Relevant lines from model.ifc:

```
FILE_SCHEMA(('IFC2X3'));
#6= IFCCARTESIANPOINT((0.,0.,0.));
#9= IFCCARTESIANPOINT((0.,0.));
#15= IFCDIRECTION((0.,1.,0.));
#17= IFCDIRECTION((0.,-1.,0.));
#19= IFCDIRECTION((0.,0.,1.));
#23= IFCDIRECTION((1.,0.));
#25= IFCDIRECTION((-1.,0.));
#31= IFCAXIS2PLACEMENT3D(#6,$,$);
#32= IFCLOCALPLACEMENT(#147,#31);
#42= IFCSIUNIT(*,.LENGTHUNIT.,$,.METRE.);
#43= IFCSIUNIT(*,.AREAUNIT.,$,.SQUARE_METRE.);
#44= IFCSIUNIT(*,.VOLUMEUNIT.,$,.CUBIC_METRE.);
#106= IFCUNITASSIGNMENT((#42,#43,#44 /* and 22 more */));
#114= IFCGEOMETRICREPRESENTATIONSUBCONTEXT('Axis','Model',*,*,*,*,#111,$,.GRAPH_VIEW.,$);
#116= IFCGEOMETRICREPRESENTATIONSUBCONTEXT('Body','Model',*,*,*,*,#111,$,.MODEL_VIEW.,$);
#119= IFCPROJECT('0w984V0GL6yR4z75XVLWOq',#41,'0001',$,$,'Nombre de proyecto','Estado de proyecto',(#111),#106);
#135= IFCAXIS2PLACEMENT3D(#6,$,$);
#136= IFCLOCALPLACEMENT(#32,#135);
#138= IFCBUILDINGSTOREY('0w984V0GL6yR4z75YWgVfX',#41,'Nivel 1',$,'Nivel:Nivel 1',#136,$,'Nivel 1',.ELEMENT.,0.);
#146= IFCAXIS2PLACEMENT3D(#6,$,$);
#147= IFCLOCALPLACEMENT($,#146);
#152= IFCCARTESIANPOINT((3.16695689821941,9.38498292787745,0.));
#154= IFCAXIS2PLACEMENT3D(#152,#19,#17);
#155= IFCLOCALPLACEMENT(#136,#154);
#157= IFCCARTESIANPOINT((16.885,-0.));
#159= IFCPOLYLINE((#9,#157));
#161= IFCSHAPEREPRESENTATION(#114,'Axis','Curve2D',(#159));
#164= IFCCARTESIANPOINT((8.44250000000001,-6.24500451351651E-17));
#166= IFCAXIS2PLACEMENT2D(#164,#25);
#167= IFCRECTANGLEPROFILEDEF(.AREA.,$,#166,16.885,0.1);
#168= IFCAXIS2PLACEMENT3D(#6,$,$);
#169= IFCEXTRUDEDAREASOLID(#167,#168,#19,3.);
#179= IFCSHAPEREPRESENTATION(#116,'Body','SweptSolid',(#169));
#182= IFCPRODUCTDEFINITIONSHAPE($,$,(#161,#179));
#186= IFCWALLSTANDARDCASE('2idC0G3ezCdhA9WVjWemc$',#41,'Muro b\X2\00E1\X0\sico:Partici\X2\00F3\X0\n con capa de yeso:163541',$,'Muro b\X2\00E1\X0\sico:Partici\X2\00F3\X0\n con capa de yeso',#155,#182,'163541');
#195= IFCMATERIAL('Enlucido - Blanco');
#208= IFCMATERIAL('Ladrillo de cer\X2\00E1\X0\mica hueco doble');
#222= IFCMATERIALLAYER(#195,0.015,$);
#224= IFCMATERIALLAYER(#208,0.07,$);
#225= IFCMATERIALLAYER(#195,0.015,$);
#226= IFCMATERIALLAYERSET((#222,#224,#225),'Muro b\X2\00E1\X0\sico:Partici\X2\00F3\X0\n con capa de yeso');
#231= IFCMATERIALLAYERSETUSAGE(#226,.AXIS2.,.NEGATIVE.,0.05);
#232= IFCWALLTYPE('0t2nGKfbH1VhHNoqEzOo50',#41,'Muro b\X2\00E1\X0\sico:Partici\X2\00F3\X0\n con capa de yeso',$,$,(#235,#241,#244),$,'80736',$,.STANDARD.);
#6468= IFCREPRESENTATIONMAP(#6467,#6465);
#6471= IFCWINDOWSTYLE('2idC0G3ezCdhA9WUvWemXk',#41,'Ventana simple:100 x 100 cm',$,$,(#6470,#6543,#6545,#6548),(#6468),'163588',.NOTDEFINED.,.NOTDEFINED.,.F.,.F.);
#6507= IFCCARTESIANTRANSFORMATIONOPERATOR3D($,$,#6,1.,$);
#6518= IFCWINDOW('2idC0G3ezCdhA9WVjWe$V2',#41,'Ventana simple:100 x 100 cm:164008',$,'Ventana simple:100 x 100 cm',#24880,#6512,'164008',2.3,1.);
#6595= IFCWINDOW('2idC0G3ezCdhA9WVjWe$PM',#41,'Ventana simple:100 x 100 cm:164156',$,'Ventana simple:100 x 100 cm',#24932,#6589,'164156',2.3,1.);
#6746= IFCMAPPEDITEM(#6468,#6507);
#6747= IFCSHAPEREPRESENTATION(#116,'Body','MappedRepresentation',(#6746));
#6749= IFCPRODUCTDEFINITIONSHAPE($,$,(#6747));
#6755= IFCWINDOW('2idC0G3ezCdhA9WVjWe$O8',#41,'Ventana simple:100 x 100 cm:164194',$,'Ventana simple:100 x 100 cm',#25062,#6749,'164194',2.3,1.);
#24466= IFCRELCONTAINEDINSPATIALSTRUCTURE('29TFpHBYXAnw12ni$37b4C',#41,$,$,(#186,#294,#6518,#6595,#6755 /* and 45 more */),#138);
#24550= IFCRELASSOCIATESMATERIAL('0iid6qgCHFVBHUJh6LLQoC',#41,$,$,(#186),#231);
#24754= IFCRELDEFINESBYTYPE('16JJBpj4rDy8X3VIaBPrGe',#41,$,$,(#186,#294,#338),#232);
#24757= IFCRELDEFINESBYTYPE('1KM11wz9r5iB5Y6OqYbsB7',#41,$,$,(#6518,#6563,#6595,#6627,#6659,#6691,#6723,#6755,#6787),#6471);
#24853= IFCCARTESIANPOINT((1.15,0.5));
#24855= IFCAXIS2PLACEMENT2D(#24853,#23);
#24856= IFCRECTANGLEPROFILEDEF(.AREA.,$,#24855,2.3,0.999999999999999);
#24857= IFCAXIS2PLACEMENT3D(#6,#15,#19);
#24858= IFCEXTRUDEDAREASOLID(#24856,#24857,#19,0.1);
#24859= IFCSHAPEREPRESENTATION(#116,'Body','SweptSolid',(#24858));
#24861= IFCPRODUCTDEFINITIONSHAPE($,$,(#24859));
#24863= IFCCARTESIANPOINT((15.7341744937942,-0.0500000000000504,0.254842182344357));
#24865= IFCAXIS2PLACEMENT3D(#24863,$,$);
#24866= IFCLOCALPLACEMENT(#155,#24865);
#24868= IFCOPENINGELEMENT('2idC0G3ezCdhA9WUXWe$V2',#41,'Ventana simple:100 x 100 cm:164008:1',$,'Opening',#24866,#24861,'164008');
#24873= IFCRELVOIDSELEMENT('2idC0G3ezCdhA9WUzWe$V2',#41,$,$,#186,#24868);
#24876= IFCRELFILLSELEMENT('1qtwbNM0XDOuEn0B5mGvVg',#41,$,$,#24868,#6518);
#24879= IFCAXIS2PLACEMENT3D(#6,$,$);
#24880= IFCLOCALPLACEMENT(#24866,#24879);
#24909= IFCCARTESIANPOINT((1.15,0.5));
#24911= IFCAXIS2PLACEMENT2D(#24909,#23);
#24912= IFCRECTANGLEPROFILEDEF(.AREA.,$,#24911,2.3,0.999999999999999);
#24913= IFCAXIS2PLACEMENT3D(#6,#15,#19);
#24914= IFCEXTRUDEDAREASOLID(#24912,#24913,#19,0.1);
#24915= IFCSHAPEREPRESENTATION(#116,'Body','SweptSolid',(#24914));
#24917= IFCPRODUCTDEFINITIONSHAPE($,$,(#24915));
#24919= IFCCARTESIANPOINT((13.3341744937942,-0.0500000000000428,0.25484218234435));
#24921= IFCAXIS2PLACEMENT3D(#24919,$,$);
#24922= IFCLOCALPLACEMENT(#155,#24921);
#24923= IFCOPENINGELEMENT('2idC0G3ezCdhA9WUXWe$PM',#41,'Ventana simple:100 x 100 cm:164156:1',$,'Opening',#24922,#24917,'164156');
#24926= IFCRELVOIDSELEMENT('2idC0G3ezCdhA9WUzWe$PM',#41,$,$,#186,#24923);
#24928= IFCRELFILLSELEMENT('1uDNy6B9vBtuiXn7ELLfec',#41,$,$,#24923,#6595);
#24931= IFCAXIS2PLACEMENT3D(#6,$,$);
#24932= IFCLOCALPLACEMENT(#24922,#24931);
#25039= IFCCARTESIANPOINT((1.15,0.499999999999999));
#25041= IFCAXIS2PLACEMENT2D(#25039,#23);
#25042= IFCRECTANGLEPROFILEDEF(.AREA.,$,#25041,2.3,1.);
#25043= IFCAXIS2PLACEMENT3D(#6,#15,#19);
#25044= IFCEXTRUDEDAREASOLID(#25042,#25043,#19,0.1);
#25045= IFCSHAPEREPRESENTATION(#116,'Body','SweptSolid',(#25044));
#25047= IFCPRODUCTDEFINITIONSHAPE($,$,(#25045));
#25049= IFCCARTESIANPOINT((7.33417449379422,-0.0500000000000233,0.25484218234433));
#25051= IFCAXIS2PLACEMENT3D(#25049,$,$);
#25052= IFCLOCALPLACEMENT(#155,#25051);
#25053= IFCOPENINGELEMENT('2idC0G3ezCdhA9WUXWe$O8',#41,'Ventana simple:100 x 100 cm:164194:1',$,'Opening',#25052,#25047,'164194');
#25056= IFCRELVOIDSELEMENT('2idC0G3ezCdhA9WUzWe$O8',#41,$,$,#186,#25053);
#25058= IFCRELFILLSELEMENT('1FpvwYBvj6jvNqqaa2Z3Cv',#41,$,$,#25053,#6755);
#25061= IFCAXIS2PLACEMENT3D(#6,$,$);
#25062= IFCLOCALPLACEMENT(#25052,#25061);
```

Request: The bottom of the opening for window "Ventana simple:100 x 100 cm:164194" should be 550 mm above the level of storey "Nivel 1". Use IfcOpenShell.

```python
import numpy as np
import ifcopenshell
import ifcopenshell.api.geometry
import ifcopenshell.geom
import ifcopenshell.util.element
import ifcopenshell.util.placement
import ifcopenshell.util.shape
import ifcopenshell.util.unit

model = ifcopenshell.open("model.ifc")
unit_scale = ifcopenshell.util.unit.calculate_unit_scale(model)

window = model.by_guid("2idC0G3ezCdhA9WVjWe$O8")
opening = window.FillsVoids[0].RelatingOpeningElement
storey = ifcopenshell.util.element.get_container(window, ifc_class="IfcBuildingStorey")
level = ifcopenshell.util.placement.get_local_placement(storey.ObjectPlacement)[2, 3]

# The opening's origin need not be at the sill, so measure its lowest point.
shape = ifcopenshell.geom.create_shape(ifcopenshell.geom.settings(), opening)
bottom = ifcopenshell.util.shape.get_shape_bottom_elevation(shape, shape.geometry) / unit_scale
dz = level + 0.55 - bottom

shift = np.array([0.0, 0.0, dz])
# The window is placed relative to its opening, so it follows when the opening moves.
matrix = ifcopenshell.util.placement.get_local_placement(opening.ObjectPlacement)
matrix[:3, 3] += shift
ifcopenshell.api.geometry.edit_object_placement(
    model, product=opening, matrix=matrix, is_si=False, should_transform_children=True
)

print(f"moved by {dz * unit_scale:+.3f} m")

model.write("model_rev.ifc")
```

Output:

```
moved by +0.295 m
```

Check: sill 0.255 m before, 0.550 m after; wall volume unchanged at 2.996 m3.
